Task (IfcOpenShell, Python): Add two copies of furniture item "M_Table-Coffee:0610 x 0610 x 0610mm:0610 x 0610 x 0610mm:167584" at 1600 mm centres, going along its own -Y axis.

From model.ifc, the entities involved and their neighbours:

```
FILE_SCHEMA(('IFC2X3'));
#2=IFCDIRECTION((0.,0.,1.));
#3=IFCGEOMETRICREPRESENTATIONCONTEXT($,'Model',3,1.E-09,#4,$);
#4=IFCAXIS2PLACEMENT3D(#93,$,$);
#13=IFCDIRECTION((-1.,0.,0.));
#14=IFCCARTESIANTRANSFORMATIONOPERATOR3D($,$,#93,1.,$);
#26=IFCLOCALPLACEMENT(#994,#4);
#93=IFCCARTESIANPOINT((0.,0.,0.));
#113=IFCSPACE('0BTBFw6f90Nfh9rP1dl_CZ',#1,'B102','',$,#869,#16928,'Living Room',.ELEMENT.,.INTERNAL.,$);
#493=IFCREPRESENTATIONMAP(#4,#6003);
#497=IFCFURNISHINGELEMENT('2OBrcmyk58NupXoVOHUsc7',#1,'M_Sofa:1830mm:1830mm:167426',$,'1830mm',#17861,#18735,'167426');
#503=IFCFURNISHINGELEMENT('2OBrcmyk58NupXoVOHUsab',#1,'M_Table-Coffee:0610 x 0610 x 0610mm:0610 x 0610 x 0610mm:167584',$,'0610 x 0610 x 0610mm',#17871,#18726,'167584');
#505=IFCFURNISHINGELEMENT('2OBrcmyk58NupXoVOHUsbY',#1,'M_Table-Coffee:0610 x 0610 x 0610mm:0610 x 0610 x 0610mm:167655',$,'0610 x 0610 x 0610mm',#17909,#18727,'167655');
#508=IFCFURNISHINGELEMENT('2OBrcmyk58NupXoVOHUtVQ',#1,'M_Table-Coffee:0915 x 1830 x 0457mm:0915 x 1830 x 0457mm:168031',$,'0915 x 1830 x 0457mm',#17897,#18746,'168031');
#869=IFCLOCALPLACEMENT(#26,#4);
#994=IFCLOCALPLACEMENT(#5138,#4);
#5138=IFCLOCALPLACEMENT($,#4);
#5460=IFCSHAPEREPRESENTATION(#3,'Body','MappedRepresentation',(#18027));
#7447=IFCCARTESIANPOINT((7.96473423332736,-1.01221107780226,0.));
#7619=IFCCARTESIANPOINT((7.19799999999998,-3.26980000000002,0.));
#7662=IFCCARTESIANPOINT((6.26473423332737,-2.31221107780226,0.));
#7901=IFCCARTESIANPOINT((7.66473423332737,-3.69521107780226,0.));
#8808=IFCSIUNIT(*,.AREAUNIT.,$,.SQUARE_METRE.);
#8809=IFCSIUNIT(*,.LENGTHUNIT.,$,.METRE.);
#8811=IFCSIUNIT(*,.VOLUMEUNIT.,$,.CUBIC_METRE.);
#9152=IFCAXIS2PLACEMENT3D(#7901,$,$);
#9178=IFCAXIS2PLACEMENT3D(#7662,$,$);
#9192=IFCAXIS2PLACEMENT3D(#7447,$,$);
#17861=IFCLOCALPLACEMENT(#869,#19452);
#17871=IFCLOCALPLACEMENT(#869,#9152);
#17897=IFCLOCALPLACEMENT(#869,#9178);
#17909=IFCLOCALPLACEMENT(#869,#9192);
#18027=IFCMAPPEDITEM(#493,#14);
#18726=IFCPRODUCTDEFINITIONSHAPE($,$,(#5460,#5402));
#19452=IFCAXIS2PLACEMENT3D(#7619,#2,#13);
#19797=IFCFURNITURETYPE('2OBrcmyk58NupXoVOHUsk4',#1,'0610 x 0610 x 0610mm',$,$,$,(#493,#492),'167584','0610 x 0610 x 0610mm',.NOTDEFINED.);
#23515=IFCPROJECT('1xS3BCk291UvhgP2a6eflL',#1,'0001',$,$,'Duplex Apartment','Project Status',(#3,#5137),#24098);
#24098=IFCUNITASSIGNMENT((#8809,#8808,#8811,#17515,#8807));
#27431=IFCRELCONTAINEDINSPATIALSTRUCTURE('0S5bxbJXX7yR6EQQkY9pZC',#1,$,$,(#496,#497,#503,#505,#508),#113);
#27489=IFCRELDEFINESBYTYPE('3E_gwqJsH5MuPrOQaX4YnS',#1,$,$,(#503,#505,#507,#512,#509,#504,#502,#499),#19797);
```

```python
import ifcopenshell
import ifcopenshell.api.geometry
import ifcopenshell.api.root
import ifcopenshell.util.element
import ifcopenshell.util.placement
import ifcopenshell.util.unit

model = ifcopenshell.open("model.ifc")
unit_scale = ifcopenshell.util.unit.calculate_unit_scale(model)


def reuse_history(source, copy):
    """copy_class also copies each property set's owner history, people and application; keep the originals."""
    for rel in copy.IsDefinedBy:
        if rel.is_a("IfcRelDefinesByProperties") and (history := rel.RelatingPropertyDefinition.OwnerHistory):
            rel.RelatingPropertyDefinition.OwnerHistory = source.OwnerHistory
            ifcopenshell.util.element.remove_deep2(model, history)


source = model.by_guid("2OBrcmyk58NupXoVOHUsab")
base = ifcopenshell.util.placement.get_local_placement(source.ObjectPlacement)
step = -base[:3, 1] * 1.6 / unit_scale

for i in range(1, 3):
    copy = ifcopenshell.api.root.copy_class(model, product=source)
    copy.Representation = ifcopenshell.util.element.copy_deep(
        model, source.Representation, exclude=["IfcGeometricRepresentationContext", "IfcRepresentationMap"]
    )
    copy.Name = "M_Table-Coffee:0610 x 0610 x 0610mm:0610 x 0610 x 0610mm"
    copy.Tag = None
    reuse_history(source, copy)
    matrix = base.copy()
    matrix[:3, 3] += i * step
    print("added at", matrix[:3, 3].round(3) + 0.0)
    ifcopenshell.api.geometry.edit_object_placement(model, product=copy, matrix=matrix, is_si=False)

model.write("model_rev.ifc")
```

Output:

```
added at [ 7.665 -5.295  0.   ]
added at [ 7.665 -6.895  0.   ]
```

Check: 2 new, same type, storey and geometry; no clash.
